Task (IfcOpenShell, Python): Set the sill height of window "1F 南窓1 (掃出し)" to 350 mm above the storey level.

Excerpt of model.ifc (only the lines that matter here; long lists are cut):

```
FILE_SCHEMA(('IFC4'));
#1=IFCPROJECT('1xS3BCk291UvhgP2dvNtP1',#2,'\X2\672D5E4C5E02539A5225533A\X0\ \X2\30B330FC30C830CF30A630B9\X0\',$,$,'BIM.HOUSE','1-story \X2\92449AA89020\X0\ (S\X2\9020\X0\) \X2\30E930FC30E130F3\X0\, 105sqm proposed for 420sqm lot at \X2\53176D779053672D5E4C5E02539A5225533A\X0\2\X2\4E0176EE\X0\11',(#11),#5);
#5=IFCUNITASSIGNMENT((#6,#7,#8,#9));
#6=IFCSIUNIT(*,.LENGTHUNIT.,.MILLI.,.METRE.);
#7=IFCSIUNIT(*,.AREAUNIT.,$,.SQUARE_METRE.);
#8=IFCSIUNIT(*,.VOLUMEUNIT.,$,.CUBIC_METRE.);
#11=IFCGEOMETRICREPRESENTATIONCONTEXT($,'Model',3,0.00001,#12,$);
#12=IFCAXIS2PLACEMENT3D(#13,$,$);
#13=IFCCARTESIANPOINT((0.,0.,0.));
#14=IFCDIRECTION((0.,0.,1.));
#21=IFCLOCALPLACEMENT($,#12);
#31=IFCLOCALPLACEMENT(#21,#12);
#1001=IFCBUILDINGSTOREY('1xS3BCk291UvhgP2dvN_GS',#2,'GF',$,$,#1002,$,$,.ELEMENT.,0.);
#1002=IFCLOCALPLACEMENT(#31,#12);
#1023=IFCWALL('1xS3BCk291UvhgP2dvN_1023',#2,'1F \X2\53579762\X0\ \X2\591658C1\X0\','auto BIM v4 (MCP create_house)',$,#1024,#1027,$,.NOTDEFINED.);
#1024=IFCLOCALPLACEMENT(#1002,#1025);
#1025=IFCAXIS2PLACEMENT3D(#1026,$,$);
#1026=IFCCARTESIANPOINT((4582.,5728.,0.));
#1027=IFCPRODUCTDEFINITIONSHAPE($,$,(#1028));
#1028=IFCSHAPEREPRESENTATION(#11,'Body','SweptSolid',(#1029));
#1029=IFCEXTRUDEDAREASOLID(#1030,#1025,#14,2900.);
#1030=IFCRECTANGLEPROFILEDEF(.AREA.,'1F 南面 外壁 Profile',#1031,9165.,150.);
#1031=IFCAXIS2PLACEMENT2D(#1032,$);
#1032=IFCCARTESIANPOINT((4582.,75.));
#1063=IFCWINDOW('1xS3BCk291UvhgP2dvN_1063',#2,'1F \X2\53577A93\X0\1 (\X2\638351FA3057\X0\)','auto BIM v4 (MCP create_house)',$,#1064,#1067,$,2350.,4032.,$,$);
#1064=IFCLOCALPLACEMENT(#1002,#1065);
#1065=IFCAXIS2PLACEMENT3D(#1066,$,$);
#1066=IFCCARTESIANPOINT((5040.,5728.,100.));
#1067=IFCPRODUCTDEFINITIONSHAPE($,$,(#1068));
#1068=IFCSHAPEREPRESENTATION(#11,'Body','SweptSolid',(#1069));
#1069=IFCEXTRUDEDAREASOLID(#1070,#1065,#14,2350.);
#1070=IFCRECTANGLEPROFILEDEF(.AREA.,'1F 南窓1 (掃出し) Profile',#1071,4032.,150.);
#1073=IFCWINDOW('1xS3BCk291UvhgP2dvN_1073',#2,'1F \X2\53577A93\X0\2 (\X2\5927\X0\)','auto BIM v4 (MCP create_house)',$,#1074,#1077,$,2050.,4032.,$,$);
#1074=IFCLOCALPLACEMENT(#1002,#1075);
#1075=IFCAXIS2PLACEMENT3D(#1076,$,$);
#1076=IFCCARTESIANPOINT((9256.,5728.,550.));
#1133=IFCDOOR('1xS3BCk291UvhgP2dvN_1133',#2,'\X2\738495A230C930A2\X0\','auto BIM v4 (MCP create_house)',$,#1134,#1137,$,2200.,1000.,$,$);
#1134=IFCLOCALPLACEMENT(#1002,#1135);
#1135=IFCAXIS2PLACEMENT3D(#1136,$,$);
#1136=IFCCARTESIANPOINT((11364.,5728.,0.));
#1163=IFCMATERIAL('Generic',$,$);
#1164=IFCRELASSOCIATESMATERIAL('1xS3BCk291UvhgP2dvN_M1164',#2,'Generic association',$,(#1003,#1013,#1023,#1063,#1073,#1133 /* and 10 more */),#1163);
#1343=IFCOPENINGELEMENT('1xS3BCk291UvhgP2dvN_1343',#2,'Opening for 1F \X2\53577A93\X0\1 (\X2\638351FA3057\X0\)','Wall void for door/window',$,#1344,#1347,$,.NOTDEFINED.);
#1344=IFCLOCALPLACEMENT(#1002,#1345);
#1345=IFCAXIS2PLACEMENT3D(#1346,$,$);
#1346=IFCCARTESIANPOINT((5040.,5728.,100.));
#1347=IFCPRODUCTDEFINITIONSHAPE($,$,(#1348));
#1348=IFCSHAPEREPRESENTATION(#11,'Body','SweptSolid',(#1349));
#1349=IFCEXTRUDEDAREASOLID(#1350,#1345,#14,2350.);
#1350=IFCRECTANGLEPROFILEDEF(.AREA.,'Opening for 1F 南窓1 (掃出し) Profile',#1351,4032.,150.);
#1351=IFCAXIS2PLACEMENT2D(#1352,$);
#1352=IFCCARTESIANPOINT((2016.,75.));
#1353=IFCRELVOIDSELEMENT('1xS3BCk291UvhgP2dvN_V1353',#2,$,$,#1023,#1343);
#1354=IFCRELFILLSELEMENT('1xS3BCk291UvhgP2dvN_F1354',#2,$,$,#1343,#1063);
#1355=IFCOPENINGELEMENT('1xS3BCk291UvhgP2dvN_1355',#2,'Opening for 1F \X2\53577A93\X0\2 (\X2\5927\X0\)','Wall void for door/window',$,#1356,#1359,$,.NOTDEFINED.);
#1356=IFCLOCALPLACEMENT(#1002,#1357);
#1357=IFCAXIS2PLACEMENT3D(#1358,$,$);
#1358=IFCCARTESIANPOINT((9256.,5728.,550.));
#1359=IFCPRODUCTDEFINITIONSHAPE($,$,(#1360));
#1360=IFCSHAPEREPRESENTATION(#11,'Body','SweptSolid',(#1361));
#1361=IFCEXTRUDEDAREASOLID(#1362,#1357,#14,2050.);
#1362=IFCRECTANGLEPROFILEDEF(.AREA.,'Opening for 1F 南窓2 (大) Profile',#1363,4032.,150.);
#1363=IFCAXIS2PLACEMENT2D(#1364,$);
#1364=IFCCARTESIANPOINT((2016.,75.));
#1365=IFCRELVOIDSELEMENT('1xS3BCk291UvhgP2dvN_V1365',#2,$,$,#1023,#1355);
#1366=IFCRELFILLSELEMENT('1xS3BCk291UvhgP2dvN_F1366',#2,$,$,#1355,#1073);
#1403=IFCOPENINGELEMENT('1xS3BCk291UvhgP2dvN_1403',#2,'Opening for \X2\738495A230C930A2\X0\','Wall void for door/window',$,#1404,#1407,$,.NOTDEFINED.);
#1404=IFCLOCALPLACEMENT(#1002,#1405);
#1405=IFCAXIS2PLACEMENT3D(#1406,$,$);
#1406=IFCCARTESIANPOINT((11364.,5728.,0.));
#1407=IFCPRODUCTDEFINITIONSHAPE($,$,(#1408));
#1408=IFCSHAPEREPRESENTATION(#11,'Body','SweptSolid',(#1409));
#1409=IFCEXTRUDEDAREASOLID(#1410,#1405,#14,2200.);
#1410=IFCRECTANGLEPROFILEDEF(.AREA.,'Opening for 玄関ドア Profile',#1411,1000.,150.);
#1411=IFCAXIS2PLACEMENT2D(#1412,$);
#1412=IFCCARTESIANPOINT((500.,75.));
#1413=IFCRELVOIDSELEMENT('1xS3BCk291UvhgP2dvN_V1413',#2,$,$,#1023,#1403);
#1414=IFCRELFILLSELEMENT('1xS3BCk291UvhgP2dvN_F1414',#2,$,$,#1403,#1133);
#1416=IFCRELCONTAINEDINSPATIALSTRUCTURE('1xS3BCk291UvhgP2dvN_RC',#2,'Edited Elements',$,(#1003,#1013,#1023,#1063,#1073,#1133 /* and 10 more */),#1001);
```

```python
import numpy as np
import ifcopenshell
import ifcopenshell.api.geometry
import ifcopenshell.geom
import ifcopenshell.util.element
import ifcopenshell.util.placement
import ifcopenshell.util.shape
import ifcopenshell.util.unit

model = ifcopenshell.open("model.ifc")
unit_scale = ifcopenshell.util.unit.calculate_unit_scale(model)

window = model.by_id(1063)
opening = window.FillsVoids[0].RelatingOpeningElement
storey = ifcopenshell.util.element.get_container(window, ifc_class="IfcBuildingStorey")
level = ifcopenshell.util.placement.get_local_placement(storey.ObjectPlacement)[2, 3]

# The opening's origin need not be at the sill, so measure its lowest point.
shape = ifcopenshell.geom.create_shape(ifcopenshell.geom.settings(), opening)
bottom = ifcopenshell.util.shape.get_shape_bottom_elevation(shape, shape.geometry) / unit_scale
dz = level + 0.35 / unit_scale - bottom

shift = np.array([0.0, 0.0, dz])
# The window is not placed relative to its opening, so move both.
for product in (opening, window):
    matrix = ifcopenshell.util.placement.get_local_placement(product.ObjectPlacement)
    matrix[:3, 3] += shift
    ifcopenshell.api.geometry.edit_object_placement(model, product=product, matrix=matrix, is_si=False)

print(f"moved by {dz * unit_scale:+.3f} m")

model.write("model-out.ifc")
```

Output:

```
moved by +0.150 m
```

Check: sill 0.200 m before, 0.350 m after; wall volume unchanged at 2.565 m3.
